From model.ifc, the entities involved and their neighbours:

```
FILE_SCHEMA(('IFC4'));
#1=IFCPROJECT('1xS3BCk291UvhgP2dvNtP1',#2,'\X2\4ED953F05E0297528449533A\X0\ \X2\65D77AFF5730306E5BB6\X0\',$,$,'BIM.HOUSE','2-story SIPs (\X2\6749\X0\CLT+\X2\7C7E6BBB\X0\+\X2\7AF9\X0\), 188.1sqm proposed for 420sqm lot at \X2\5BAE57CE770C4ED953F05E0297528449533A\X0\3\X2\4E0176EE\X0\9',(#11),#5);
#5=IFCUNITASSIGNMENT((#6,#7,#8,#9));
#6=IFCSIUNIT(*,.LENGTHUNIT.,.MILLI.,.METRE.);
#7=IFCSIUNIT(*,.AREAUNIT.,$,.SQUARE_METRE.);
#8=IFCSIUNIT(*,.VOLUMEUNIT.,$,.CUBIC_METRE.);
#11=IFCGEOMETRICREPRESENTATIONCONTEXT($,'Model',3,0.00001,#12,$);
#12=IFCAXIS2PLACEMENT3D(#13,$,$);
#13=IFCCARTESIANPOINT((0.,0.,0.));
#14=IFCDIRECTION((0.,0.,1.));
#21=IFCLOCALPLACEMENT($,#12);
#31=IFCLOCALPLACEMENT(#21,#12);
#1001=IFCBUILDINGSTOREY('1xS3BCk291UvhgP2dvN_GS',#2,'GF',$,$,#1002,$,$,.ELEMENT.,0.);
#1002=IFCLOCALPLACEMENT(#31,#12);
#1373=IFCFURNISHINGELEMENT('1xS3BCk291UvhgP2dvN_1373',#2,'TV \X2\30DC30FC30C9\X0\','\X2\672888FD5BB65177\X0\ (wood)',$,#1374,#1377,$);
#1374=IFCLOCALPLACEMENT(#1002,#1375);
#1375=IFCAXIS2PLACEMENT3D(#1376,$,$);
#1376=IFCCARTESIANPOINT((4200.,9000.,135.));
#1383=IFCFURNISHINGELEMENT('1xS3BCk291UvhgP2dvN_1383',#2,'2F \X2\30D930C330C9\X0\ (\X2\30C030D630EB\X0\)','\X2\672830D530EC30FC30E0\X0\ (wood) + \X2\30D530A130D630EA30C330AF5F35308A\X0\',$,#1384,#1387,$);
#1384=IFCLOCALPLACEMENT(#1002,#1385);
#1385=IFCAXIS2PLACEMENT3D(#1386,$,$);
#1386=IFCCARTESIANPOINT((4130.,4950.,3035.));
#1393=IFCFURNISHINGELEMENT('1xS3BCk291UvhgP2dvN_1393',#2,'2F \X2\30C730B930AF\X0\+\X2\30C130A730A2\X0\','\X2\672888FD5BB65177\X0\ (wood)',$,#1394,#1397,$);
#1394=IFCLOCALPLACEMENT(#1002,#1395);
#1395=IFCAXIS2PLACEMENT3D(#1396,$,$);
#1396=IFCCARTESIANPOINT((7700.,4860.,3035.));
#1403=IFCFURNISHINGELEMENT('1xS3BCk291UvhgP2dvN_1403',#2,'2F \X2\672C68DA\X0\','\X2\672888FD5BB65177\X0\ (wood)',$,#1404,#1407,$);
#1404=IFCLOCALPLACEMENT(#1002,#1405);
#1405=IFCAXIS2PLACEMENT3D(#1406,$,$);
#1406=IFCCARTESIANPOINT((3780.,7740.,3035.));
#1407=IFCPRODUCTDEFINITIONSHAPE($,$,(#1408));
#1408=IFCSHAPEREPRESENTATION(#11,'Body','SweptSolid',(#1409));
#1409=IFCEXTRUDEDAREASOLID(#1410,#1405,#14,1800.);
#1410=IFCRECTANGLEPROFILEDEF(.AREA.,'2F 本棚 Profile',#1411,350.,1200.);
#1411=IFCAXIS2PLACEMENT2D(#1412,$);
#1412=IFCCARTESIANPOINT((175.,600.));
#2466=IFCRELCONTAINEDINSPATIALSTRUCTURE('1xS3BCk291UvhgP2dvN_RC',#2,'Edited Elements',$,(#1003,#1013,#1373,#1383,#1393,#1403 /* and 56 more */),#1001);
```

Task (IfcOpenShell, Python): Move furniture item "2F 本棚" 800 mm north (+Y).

```python
import ifcopenshell
import ifcopenshell.api.geometry
import ifcopenshell.util.placement
import ifcopenshell.util.unit

model = ifcopenshell.open("model.ifc")
unit_scale = ifcopenshell.util.unit.calculate_unit_scale(model)

item = model.by_guid("1xS3BCk291UvhgP2dvN_1403")
matrix = ifcopenshell.util.placement.get_local_placement(item.ObjectPlacement)
matrix[1, 3] += 0.8 / unit_scale
ifcopenshell.api.geometry.edit_object_placement(model, product=item, matrix=matrix, is_si=False)

print(ifcopenshell.util.placement.get_local_placement(item.ObjectPlacement).round(3) + 0.0)

model.write("model_updated.ifc")
```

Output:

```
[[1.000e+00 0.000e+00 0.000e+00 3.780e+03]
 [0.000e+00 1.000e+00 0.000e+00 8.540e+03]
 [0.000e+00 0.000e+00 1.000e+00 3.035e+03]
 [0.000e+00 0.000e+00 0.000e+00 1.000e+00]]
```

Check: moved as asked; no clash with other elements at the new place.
